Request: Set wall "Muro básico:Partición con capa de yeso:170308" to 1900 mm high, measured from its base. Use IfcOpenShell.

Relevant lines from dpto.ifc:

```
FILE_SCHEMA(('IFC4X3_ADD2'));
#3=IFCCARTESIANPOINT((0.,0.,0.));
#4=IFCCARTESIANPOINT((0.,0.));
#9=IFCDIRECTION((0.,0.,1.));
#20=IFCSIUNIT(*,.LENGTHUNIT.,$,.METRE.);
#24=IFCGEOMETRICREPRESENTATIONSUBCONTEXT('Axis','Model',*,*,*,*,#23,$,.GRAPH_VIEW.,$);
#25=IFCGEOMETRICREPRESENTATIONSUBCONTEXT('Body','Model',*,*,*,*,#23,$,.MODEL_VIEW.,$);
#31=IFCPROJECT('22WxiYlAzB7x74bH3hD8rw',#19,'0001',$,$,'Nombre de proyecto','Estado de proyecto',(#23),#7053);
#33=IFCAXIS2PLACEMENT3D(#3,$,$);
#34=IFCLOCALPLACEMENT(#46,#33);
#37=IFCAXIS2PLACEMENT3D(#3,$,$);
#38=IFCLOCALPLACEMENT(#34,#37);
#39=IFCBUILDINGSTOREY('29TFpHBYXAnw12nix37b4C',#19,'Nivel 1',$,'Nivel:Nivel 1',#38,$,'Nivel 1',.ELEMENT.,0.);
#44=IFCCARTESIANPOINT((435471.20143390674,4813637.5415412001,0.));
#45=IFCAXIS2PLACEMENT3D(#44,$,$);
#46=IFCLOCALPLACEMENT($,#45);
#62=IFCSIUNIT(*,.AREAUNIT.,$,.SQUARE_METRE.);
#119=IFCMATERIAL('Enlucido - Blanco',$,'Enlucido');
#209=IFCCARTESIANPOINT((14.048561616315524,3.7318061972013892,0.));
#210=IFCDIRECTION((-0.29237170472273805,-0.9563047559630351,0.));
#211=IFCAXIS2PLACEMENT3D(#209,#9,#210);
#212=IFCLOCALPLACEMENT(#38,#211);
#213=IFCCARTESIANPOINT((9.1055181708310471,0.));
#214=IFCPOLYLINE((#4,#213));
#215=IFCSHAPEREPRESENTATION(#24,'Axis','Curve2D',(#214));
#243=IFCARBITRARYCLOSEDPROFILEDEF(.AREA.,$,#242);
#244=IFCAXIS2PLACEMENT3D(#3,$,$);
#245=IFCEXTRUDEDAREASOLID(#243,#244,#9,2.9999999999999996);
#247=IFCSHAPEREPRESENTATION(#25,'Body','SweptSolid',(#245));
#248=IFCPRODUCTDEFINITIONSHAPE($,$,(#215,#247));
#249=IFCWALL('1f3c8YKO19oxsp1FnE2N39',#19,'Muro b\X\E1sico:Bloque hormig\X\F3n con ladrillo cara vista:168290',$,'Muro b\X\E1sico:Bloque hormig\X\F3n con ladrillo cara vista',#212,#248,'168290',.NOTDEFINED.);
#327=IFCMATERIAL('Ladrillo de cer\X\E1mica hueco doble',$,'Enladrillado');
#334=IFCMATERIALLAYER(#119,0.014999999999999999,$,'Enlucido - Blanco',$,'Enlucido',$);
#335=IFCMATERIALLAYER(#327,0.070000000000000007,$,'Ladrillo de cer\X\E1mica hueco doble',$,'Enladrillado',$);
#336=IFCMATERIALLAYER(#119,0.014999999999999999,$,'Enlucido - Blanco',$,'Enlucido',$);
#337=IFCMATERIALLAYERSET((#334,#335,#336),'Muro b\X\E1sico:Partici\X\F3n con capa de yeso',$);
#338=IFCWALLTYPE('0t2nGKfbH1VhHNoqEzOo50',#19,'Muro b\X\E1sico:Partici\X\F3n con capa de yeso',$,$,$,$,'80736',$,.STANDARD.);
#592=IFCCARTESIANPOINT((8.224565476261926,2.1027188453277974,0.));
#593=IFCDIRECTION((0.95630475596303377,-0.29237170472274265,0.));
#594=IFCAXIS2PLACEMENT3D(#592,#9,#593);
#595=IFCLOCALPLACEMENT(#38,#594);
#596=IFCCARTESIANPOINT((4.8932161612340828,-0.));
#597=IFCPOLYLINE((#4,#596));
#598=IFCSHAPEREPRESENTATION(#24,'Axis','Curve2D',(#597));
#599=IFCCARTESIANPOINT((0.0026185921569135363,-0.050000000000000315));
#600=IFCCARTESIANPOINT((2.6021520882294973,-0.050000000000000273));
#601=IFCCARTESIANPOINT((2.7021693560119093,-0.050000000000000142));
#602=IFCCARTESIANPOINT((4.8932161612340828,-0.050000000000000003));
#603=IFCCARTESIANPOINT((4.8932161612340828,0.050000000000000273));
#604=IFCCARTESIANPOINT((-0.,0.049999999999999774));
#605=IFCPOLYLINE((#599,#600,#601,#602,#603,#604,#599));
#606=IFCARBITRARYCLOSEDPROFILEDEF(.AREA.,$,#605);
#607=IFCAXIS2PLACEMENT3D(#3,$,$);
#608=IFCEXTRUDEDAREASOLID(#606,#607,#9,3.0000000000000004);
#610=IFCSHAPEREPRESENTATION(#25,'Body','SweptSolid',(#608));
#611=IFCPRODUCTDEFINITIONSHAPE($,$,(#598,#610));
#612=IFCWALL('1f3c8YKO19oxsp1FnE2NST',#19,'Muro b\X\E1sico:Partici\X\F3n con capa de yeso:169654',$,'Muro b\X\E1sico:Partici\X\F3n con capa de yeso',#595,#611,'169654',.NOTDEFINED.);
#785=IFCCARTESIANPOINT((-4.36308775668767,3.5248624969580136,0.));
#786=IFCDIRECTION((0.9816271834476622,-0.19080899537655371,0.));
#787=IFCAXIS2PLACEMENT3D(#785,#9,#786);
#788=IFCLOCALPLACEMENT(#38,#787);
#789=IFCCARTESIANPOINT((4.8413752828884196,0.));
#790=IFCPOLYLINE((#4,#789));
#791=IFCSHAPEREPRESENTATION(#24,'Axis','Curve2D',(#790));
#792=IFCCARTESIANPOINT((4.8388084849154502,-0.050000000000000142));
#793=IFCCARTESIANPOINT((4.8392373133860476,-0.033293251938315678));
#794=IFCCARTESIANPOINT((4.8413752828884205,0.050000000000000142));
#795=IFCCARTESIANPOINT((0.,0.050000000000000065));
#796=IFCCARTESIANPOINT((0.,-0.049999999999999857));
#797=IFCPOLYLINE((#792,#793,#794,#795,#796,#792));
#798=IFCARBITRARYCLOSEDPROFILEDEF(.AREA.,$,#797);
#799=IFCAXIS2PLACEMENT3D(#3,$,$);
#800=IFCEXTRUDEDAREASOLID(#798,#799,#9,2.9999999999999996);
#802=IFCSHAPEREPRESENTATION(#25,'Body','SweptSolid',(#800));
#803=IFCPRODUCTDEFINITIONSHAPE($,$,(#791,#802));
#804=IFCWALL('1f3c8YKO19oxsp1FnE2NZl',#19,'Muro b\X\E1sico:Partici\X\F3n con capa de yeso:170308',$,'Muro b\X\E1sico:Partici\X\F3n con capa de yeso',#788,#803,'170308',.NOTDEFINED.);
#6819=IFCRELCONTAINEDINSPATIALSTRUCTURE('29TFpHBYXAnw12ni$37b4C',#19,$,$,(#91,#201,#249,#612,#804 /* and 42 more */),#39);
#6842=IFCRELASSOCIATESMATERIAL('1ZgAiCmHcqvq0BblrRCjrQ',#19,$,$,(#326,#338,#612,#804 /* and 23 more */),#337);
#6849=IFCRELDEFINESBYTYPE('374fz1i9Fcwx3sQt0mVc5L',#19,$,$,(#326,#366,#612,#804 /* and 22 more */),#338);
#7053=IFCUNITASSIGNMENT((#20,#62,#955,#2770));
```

```python
import ifcopenshell
import ifcopenshell.geom
import ifcopenshell.util.representation
import ifcopenshell.util.shape

model = ifcopenshell.open("dpto.ifc")
settings = ifcopenshell.geom.settings()


def volume(element):
    """Net volume in cubic metres, openings subtracted."""
    shape = ifcopenshell.geom.create_shape(settings, element)
    return ifcopenshell.util.shape.get_volume(shape.geometry)


wall = model.by_id(804)
before = volume(wall)

body = ifcopenshell.util.representation.get_representation(wall, "Model", "Body")
solid = body.Items[0]
old_height = solid.Depth
solid.Depth = 1.9
after = volume(wall)

print(f"height {old_height:g} -> {solid.Depth:g}, volume {before:.3f} -> {after:.3f} m3")

model.write("dpto-out.ifc")
```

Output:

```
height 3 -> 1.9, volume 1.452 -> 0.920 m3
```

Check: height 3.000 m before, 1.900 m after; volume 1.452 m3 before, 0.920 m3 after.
